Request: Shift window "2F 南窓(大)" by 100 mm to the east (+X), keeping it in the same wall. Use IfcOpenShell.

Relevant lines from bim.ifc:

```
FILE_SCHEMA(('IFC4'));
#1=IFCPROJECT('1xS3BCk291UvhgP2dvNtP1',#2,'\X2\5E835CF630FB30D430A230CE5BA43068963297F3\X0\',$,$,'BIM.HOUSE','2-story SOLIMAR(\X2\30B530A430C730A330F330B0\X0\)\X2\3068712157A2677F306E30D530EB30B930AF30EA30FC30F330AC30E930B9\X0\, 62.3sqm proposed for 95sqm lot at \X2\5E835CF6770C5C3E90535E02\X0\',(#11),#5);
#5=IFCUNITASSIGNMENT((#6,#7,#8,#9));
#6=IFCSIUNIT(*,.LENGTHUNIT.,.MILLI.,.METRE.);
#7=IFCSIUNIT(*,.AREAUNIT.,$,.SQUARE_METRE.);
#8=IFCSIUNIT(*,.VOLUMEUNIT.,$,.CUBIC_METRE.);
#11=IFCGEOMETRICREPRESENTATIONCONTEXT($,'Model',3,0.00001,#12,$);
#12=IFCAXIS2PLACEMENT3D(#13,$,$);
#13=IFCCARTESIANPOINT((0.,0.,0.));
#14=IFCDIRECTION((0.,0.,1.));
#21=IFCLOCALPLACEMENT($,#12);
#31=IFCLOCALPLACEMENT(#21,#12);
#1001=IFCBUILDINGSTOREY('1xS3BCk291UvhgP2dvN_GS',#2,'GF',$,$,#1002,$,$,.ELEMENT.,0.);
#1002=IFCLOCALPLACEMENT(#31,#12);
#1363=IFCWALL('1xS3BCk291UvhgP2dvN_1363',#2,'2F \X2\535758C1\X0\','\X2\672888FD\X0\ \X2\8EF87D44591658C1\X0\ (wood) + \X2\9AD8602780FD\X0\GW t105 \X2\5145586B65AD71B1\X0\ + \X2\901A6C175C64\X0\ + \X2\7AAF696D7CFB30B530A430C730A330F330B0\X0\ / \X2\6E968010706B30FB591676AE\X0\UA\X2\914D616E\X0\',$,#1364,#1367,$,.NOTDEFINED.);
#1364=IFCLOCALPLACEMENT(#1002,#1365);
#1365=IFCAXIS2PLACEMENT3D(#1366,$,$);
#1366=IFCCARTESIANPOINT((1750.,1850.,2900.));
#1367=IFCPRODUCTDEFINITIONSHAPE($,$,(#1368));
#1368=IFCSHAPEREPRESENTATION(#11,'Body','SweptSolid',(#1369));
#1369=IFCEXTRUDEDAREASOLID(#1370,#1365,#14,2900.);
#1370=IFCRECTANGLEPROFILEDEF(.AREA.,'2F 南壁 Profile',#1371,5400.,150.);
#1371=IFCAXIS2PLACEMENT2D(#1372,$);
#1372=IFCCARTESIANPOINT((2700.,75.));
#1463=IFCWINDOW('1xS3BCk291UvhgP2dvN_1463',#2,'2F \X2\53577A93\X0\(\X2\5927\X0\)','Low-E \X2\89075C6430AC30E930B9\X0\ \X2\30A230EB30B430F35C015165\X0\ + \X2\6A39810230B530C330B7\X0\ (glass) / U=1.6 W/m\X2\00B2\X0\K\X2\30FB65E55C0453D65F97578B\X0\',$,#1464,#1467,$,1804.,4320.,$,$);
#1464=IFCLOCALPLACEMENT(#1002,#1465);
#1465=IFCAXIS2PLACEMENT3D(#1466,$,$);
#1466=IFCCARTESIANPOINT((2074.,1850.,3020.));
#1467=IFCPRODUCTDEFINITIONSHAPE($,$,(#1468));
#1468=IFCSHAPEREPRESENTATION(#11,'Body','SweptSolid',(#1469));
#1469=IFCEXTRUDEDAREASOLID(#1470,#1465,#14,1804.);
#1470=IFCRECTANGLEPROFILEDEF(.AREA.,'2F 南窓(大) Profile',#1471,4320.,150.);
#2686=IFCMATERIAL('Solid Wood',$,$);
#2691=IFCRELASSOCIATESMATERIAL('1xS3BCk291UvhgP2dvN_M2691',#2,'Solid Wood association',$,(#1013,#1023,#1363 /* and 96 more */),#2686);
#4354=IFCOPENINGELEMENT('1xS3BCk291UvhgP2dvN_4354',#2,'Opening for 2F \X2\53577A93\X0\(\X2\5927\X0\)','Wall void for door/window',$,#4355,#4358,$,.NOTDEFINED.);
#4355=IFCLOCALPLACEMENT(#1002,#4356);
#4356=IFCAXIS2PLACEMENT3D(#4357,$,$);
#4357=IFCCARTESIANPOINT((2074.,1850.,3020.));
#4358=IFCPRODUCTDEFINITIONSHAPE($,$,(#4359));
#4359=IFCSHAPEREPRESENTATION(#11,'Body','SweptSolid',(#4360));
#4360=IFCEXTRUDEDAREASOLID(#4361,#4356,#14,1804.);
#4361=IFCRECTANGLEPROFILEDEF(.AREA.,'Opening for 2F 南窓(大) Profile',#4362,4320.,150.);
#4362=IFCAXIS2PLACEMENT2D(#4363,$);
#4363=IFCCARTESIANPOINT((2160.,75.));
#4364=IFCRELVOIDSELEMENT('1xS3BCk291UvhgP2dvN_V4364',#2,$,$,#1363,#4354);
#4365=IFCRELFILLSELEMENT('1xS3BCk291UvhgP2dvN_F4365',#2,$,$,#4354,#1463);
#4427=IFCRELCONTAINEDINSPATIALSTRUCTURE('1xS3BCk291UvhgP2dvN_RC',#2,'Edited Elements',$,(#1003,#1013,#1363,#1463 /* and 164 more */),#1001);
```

```python
import ifcopenshell
import ifcopenshell.api.geometry
import ifcopenshell.util.placement
import ifcopenshell.util.unit

model = ifcopenshell.open("bim.ifc")
unit_scale = ifcopenshell.util.unit.calculate_unit_scale(model)

window = model.by_guid("1xS3BCk291UvhgP2dvN_1463")
opening = window.FillsVoids[0].RelatingOpeningElement
wall = opening.VoidsElements[0].RelatingBuildingElement

wall_matrix = ifcopenshell.util.placement.get_local_placement(wall.ObjectPlacement)
shift = wall_matrix[:3, 0] * 0.1 / unit_scale
before = ifcopenshell.util.placement.get_local_placement(window.ObjectPlacement)[:3, 3].copy()

# The window is not placed relative to its opening, so move both.
for product in (opening, window):
    matrix = ifcopenshell.util.placement.get_local_placement(product.ObjectPlacement)
    matrix[:3, 3] += shift
    ifcopenshell.api.geometry.edit_object_placement(model, product=product, matrix=matrix, is_si=False)

after = ifcopenshell.util.placement.get_local_placement(window.ObjectPlacement)[:3, 3]
print("window moved by", (after - before).round(3) + 0.0)

model.write("bim_rev.ifc")
```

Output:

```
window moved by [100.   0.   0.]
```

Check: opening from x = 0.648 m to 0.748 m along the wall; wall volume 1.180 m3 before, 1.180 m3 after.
